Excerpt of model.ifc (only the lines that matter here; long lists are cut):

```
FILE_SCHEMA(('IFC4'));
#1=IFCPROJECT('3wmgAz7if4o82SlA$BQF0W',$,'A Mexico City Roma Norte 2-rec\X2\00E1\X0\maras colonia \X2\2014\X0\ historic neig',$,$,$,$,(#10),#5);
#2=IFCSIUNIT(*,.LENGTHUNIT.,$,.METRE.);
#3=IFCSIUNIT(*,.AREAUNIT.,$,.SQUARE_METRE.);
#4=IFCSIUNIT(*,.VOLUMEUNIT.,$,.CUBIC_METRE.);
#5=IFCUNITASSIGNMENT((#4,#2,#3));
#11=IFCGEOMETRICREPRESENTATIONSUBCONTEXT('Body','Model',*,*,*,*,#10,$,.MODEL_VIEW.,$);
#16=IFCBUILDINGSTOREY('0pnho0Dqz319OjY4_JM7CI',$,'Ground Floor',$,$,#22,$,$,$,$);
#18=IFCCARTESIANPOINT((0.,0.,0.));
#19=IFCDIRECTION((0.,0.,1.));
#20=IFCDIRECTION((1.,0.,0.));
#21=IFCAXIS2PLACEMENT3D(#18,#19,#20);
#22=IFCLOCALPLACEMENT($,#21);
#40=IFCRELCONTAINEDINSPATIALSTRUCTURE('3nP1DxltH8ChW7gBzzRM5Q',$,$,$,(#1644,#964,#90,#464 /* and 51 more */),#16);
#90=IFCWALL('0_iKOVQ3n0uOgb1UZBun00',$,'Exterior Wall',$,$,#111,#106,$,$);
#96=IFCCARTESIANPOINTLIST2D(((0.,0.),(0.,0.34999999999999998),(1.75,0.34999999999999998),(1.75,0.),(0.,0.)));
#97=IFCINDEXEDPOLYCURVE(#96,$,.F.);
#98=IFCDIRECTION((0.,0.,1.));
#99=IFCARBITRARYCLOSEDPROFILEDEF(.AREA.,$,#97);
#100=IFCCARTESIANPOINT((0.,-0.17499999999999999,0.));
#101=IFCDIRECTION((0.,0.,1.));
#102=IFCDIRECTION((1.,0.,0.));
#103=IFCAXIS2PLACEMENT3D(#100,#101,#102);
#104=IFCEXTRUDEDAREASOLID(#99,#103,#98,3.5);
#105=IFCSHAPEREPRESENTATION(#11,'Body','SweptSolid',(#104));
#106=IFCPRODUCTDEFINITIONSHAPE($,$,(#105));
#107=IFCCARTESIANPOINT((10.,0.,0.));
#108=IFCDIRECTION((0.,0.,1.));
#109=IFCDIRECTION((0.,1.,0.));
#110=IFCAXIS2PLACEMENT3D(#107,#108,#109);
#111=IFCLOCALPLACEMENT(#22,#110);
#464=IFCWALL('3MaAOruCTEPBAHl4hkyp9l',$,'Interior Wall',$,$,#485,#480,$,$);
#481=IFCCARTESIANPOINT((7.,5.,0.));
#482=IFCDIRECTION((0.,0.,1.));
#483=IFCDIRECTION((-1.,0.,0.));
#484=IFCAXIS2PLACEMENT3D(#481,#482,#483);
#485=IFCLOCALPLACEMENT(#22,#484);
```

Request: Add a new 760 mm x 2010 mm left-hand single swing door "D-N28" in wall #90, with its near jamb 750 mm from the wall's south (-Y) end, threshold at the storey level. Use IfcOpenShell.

```python
import numpy as np
import ifcopenshell
import ifcopenshell.api.feature
import ifcopenshell.api.geometry
import ifcopenshell.api.root
import ifcopenshell.api.spatial
import ifcopenshell.geom
import ifcopenshell.util.element
import ifcopenshell.util.placement
import ifcopenshell.util.representation
import ifcopenshell.util.shape
import ifcopenshell.util.unit

model = ifcopenshell.open("model.ifc")
unit_scale = ifcopenshell.util.unit.calculate_unit_scale(model)
settings = ifcopenshell.geom.settings()


def volume(element):
    """Net volume in cubic metres, openings subtracted."""
    shape = ifcopenshell.geom.create_shape(settings, element)
    return ifcopenshell.util.shape.get_volume(shape.geometry)


wall = model.by_id(90)
storey = ifcopenshell.util.element.get_container(wall, ifc_class="IfcBuildingStorey")
context = ifcopenshell.util.representation.get_context(model, "Model", "Body", "MODEL_VIEW")
before = volume(wall)

width, height, from_end, sill = 0.76, 2.01, 0.75, 0.0  # metres

# The wall runs along its own X axis, and the end named is its -X end.
wall_shape = ifcopenshell.geom.create_shape(settings, wall)
x, y, z = ifcopenshell.util.shape.get_vertices(wall_shape.geometry).T
start = x.min() + from_end
face, thickness = float(y.min()), float(y.max() - y.min())
wall_matrix = ifcopenshell.util.placement.get_local_placement(wall.ObjectPlacement)
level = ifcopenshell.util.placement.get_local_placement(storey.ObjectPlacement)[2, 3]


def in_wall(x, y):
    """Placement at x, y metres in the wall's axes, at sill height."""
    matrix = wall_matrix.copy()
    matrix[:, 3] = wall_matrix @ np.array([x / unit_scale, y / unit_scale, 0.0, 1.0])
    matrix[2, 3] = level + sill / unit_scale
    return matrix


# Opening: a box that overshoots both wall faces by 50 mm.
opening = ifcopenshell.api.root.create_entity(model, ifc_class="IfcOpeningElement", predefined_type="OPENING")
box = ifcopenshell.api.geometry.add_wall_representation(
    model, context=context, length=width, height=height, thickness=thickness + 0.1
)
ifcopenshell.api.geometry.assign_representation(model, product=opening, representation=box)
ifcopenshell.api.geometry.edit_object_placement(model, product=opening, matrix=in_wall(start, face - 0.05), is_si=False)
ifcopenshell.api.feature.add_feature(model, feature=opening, element=wall)

door = ifcopenshell.api.root.create_entity(model, ifc_class="IfcDoor", name="D-N28", predefined_type="DOOR")
door.OverallWidth, door.OverallHeight = width / unit_scale, height / unit_scale
door.OperationType = "SINGLE_SWING_LEFT"
body = ifcopenshell.api.geometry.add_door_representation(
    model,
    context=context,
    overall_width=door.OverallWidth,
    overall_height=door.OverallHeight,
    operation_type="SINGLE_SWING_LEFT",
    lining_properties={"LiningDepth": thickness / unit_scale, "ThresholdDepth": thickness / unit_scale},
)
ifcopenshell.api.geometry.assign_representation(model, product=door, representation=body)
ifcopenshell.api.spatial.assign_container(model, products=[door], relating_structure=storey)
ifcopenshell.api.feature.add_filling(model, opening=opening, element=door)

# The lining spans the wall, so the door starts at the wall face.
ifcopenshell.api.geometry.edit_object_placement(model, product=door, matrix=in_wall(start, face), is_si=False)

after = volume(wall)

print(f"wall volume {before:.3f} -> {after:.3f} m3")

model.write("model_rev.ifc")
```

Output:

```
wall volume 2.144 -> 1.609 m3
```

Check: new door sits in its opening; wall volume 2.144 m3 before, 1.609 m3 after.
